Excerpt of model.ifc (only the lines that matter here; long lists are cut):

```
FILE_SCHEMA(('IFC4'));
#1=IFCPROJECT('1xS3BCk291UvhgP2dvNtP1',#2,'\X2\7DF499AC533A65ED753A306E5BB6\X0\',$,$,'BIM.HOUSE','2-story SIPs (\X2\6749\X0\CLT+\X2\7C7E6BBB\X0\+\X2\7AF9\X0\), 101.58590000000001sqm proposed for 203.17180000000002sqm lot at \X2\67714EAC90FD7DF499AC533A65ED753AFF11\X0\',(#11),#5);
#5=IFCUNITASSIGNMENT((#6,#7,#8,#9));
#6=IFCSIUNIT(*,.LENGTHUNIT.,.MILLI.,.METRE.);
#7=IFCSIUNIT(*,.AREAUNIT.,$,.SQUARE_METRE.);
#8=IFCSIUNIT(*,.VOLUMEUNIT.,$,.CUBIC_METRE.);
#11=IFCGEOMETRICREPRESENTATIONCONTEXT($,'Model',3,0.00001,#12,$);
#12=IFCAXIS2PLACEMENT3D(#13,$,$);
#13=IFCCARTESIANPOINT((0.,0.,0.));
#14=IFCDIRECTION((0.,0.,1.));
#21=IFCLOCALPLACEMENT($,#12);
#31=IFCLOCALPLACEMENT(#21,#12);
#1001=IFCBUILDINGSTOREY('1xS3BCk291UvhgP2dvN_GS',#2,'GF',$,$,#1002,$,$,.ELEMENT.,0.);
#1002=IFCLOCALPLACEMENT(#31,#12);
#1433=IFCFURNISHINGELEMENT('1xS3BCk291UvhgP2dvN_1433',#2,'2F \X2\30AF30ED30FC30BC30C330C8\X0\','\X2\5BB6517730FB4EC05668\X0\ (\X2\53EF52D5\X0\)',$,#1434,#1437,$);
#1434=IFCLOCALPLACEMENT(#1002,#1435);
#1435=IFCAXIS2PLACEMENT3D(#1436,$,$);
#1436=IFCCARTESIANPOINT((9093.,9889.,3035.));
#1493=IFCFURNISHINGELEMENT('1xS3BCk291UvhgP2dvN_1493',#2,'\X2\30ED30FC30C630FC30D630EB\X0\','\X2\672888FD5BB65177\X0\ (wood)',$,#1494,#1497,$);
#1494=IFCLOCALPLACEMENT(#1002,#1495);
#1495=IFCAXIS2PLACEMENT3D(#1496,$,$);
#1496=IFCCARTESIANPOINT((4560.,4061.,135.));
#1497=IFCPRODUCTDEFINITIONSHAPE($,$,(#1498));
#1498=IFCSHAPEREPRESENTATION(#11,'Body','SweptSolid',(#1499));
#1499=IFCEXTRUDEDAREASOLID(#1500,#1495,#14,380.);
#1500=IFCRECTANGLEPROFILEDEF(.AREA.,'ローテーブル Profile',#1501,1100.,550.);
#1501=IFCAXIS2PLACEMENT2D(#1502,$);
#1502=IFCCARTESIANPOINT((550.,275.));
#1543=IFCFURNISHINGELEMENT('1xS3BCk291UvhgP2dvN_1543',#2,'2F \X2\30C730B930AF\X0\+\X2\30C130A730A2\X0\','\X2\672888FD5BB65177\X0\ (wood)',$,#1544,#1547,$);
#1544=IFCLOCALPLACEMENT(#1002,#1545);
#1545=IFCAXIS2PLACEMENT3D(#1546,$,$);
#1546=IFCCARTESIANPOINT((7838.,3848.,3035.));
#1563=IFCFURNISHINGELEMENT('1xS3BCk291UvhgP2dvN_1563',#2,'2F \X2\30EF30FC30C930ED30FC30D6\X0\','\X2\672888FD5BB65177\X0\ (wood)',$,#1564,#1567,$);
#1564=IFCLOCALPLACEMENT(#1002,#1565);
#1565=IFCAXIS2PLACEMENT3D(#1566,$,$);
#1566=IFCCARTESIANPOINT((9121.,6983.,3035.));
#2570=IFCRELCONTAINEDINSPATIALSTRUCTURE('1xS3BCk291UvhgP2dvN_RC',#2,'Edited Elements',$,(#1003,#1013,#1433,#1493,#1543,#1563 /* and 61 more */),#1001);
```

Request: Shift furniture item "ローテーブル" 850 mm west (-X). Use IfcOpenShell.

```python
import ifcopenshell
import ifcopenshell.api.geometry
import ifcopenshell.util.placement

model = ifcopenshell.open("model.ifc")

item = model.by_guid("1xS3BCk291UvhgP2dvN_1493")
matrix = ifcopenshell.util.placement.get_local_placement(item.ObjectPlacement)
matrix[0, 3] -= 850.0
ifcopenshell.api.geometry.edit_object_placement(model, product=item, matrix=matrix, is_si=False)

print(ifcopenshell.util.placement.get_local_placement(item.ObjectPlacement).round(3) + 0.0)

model.write("model_rev.ifc")
```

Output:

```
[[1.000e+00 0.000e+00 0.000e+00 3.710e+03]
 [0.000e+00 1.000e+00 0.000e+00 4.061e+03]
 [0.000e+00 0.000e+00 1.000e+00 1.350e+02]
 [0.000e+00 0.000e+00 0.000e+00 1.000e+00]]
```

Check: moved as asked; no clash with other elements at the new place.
